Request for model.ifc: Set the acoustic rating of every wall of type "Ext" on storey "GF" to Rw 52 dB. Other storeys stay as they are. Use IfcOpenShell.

First a look at what the model holds.

```python
import ifcopenshell
import ifcopenshell.util.element

model = ifcopenshell.open("model.ifc")
print(model.schema)
storey = next(s for s in model.by_type("IfcBuildingStorey") if s.Name == "GF")
walls = [e for e in ifcopenshell.util.element.get_decomposition(storey) if e.is_a("IfcWall")]
seen = {}
for e in walls:
    element_type = ifcopenshell.util.element.get_type(e)
    key = (element_type.Name if element_type != e and element_type else None, ifcopenshell.util.element.get_pset(e, "Pset_WallCommon", "AcousticRating"))
    seen[key] = seen.get(key, 0) + 1
for (name, value), count in sorted(seen.items(), key=str):
    print(count, "x", name, "|", value)
```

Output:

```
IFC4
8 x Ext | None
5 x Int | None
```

```python
import ifcopenshell
import ifcopenshell.api.pset
import ifcopenshell.util.element

model = ifcopenshell.open("model.ifc")

storey = next(s for s in model.by_type("IfcBuildingStorey") if s.Name == "GF")
walls = [e for e in ifcopenshell.util.element.get_decomposition(storey) if e.is_a("IfcWall")]

count = 0
for e in walls:
    element_type = ifcopenshell.util.element.get_type(e)
    if element_type in (None, e) or element_type.Name != "Ext":
        continue
    # add_pset returns the element's existing set when there is one.
    pset = ifcopenshell.api.pset.add_pset(model, product=e, name="Pset_WallCommon")
    ifcopenshell.api.pset.edit_pset(model, pset=pset, properties={"AcousticRating": "Rw 52 dB"})
    count += 1

print(count, "walls updated")

model.write("model_updated.ifc")
```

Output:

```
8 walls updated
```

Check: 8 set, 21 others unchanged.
